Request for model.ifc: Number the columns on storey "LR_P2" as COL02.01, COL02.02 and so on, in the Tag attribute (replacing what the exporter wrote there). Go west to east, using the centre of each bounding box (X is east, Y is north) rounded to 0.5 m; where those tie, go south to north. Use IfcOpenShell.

First a look at what the model holds.

```python
import ifcopenshell
import ifcopenshell.util.element
import ifcopenshell.util.placement

model = ifcopenshell.open("model.ifc")
print(model.schema)
storey = next(s for s in model.by_type("IfcBuildingStorey") if s.Name == "LR_P2")
columns = [e for e in ifcopenshell.util.element.get_decomposition(storey) if e.is_a("IfcColumn")]
for e in sorted(columns, key=lambda e: e.id()):
    origin = ifcopenshell.util.placement.get_local_placement(e.ObjectPlacement)[:3, 3]
    print(e.id(), e.Tag, e.Name, origin.round(2) + 0.0, sep=" | ")
```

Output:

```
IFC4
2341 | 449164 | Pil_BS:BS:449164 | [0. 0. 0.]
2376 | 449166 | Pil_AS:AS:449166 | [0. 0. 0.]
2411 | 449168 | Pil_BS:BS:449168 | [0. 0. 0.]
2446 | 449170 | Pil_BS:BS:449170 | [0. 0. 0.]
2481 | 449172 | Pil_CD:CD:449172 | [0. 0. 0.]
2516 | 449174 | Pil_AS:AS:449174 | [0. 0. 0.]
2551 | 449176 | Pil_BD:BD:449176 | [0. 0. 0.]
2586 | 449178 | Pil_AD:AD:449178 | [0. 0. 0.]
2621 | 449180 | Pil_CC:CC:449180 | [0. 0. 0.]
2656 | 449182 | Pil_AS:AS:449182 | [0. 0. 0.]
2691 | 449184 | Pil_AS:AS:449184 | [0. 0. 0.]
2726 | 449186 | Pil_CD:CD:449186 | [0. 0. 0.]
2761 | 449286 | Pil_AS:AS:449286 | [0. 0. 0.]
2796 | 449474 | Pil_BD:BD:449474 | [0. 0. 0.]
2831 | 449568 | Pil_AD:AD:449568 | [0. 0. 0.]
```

```python
import ifcopenshell
import ifcopenshell.geom
import ifcopenshell.util.element
import ifcopenshell.util.shape

model = ifcopenshell.open("model.ifc")
settings = ifcopenshell.geom.settings()
settings.set("use-world-coords", True)


def centre(element):
    shape = ifcopenshell.geom.create_shape(settings, element)
    return ifcopenshell.util.shape.get_bbox_centroid(shape.geometry)


storey = next(s for s in model.by_type("IfcBuildingStorey") if s.Name == "LR_P2")
columns = [e for e in ifcopenshell.util.element.get_decomposition(storey) if e.is_a("IfcColumn")]

# Insertion points can sit at a corner or the storey origin, so sort by the geometry (in metres).
centres = {e: centre(e) for e in columns}
columns.sort(key=lambda e: (round(centres[e][0] / 0.5), centres[e][1]))

for i, e in enumerate(columns, start=1):
    number = f"COL02.{i:02d}"
    e.Tag = number
    print(e.id(), number)

model.write("model_updated.ifc")
```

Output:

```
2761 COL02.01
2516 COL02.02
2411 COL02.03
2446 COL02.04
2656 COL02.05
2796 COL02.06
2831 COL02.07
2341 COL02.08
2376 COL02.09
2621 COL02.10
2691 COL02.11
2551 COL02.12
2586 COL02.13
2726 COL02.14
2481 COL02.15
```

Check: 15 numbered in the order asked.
